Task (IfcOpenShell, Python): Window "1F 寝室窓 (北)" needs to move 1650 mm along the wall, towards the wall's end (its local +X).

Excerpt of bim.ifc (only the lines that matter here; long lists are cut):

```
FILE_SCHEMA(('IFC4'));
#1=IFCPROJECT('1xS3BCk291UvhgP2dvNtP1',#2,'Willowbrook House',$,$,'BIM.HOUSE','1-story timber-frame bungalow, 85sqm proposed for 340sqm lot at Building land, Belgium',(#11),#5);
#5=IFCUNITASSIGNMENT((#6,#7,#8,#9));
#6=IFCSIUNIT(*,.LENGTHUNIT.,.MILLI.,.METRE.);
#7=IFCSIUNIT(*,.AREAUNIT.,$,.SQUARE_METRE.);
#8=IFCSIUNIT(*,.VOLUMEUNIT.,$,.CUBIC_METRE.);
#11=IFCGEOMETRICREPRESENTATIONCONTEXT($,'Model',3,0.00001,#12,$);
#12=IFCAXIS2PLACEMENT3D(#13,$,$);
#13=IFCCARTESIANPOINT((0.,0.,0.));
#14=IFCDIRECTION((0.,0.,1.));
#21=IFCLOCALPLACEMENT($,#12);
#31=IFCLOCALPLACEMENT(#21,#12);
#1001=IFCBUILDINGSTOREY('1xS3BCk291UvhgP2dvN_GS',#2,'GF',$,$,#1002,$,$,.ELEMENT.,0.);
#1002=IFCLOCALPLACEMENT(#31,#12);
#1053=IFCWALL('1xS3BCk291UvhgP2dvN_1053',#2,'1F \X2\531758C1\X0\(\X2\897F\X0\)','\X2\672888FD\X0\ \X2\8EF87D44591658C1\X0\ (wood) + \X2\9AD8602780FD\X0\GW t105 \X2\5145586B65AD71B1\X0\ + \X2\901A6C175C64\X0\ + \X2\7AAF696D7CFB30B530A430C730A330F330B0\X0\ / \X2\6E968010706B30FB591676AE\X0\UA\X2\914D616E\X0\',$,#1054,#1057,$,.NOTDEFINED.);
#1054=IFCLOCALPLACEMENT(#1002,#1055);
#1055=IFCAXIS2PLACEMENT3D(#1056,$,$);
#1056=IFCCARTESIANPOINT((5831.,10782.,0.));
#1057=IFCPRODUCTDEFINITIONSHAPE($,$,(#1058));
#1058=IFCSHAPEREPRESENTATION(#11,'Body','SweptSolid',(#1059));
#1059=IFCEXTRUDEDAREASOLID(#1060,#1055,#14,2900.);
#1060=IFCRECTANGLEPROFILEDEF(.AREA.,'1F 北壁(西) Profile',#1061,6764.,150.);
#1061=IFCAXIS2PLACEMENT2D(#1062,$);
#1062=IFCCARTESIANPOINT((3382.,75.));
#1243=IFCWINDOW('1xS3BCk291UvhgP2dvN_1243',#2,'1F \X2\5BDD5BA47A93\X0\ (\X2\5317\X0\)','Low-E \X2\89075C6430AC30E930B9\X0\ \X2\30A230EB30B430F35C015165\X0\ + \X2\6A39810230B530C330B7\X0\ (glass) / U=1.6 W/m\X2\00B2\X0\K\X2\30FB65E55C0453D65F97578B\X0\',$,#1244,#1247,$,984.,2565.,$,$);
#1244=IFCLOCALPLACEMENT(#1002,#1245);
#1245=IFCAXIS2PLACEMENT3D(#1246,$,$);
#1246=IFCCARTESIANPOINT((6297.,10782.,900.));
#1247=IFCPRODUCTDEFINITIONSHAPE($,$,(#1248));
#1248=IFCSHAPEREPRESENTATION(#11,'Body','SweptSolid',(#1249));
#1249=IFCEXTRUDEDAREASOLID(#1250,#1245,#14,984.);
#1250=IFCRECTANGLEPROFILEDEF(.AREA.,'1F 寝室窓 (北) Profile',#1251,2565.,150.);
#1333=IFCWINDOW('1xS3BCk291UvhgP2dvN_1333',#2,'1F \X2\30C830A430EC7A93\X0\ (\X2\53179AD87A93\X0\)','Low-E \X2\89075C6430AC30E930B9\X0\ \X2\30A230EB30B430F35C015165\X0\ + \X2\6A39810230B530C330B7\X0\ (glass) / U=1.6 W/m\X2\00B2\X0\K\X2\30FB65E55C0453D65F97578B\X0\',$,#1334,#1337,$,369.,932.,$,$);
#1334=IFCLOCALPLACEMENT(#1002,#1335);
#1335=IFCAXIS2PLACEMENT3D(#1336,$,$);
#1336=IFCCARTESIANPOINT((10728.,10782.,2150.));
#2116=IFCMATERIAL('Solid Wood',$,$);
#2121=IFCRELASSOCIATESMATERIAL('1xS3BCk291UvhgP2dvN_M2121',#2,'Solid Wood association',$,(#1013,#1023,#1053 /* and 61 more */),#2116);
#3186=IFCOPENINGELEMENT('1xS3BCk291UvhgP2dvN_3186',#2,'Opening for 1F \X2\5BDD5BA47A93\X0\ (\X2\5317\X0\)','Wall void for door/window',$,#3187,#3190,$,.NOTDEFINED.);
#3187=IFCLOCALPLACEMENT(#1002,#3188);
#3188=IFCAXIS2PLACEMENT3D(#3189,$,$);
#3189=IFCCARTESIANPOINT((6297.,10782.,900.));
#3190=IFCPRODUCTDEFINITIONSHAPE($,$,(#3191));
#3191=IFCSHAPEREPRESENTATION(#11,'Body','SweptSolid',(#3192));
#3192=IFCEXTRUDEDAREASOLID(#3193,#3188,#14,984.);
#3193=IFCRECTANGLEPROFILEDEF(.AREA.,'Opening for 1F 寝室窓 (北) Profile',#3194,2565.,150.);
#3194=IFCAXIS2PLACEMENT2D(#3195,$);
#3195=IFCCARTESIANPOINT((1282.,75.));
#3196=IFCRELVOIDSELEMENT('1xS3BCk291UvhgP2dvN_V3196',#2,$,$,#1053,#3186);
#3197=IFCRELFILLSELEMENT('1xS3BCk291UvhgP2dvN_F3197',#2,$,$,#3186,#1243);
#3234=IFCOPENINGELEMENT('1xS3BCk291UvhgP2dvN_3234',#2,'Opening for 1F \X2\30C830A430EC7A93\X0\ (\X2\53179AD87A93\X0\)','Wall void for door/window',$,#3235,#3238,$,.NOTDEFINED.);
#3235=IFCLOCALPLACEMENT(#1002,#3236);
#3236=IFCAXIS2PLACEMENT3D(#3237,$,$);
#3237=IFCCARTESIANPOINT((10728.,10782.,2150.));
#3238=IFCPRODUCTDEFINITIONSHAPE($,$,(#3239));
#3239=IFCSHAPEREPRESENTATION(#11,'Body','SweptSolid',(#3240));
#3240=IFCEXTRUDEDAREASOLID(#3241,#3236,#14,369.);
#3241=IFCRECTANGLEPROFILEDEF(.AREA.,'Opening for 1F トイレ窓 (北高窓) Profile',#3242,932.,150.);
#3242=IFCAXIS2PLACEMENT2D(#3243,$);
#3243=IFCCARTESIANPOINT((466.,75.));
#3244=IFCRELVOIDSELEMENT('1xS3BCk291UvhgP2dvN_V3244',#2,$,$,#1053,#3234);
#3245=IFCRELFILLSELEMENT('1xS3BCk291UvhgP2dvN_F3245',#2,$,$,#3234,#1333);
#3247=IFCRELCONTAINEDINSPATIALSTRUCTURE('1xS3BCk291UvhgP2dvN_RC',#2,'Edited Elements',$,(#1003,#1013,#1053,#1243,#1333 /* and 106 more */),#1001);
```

```python
import ifcopenshell
import ifcopenshell.api.geometry
import ifcopenshell.util.placement

model = ifcopenshell.open("bim.ifc")

window = model.by_guid("1xS3BCk291UvhgP2dvN_1243")
opening = window.FillsVoids[0].RelatingOpeningElement
wall = opening.VoidsElements[0].RelatingBuildingElement

wall_matrix = ifcopenshell.util.placement.get_local_placement(wall.ObjectPlacement)
shift = wall_matrix[:3, 0] * 1650.0
before = ifcopenshell.util.placement.get_local_placement(window.ObjectPlacement)[:3, 3].copy()

# The window is not placed relative to its opening, so move both.
for product in (opening, window):
    matrix = ifcopenshell.util.placement.get_local_placement(product.ObjectPlacement)
    matrix[:3, 3] += shift
    ifcopenshell.api.geometry.edit_object_placement(model, product=product, matrix=matrix, is_si=False)

after = ifcopenshell.util.placement.get_local_placement(window.ObjectPlacement)[:3, 3]
print("window moved by", (after - before).round(3) + 0.0)

model.write("bim_rev.ifc")
```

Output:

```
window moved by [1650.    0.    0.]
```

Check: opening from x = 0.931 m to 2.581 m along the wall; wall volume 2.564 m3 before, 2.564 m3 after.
